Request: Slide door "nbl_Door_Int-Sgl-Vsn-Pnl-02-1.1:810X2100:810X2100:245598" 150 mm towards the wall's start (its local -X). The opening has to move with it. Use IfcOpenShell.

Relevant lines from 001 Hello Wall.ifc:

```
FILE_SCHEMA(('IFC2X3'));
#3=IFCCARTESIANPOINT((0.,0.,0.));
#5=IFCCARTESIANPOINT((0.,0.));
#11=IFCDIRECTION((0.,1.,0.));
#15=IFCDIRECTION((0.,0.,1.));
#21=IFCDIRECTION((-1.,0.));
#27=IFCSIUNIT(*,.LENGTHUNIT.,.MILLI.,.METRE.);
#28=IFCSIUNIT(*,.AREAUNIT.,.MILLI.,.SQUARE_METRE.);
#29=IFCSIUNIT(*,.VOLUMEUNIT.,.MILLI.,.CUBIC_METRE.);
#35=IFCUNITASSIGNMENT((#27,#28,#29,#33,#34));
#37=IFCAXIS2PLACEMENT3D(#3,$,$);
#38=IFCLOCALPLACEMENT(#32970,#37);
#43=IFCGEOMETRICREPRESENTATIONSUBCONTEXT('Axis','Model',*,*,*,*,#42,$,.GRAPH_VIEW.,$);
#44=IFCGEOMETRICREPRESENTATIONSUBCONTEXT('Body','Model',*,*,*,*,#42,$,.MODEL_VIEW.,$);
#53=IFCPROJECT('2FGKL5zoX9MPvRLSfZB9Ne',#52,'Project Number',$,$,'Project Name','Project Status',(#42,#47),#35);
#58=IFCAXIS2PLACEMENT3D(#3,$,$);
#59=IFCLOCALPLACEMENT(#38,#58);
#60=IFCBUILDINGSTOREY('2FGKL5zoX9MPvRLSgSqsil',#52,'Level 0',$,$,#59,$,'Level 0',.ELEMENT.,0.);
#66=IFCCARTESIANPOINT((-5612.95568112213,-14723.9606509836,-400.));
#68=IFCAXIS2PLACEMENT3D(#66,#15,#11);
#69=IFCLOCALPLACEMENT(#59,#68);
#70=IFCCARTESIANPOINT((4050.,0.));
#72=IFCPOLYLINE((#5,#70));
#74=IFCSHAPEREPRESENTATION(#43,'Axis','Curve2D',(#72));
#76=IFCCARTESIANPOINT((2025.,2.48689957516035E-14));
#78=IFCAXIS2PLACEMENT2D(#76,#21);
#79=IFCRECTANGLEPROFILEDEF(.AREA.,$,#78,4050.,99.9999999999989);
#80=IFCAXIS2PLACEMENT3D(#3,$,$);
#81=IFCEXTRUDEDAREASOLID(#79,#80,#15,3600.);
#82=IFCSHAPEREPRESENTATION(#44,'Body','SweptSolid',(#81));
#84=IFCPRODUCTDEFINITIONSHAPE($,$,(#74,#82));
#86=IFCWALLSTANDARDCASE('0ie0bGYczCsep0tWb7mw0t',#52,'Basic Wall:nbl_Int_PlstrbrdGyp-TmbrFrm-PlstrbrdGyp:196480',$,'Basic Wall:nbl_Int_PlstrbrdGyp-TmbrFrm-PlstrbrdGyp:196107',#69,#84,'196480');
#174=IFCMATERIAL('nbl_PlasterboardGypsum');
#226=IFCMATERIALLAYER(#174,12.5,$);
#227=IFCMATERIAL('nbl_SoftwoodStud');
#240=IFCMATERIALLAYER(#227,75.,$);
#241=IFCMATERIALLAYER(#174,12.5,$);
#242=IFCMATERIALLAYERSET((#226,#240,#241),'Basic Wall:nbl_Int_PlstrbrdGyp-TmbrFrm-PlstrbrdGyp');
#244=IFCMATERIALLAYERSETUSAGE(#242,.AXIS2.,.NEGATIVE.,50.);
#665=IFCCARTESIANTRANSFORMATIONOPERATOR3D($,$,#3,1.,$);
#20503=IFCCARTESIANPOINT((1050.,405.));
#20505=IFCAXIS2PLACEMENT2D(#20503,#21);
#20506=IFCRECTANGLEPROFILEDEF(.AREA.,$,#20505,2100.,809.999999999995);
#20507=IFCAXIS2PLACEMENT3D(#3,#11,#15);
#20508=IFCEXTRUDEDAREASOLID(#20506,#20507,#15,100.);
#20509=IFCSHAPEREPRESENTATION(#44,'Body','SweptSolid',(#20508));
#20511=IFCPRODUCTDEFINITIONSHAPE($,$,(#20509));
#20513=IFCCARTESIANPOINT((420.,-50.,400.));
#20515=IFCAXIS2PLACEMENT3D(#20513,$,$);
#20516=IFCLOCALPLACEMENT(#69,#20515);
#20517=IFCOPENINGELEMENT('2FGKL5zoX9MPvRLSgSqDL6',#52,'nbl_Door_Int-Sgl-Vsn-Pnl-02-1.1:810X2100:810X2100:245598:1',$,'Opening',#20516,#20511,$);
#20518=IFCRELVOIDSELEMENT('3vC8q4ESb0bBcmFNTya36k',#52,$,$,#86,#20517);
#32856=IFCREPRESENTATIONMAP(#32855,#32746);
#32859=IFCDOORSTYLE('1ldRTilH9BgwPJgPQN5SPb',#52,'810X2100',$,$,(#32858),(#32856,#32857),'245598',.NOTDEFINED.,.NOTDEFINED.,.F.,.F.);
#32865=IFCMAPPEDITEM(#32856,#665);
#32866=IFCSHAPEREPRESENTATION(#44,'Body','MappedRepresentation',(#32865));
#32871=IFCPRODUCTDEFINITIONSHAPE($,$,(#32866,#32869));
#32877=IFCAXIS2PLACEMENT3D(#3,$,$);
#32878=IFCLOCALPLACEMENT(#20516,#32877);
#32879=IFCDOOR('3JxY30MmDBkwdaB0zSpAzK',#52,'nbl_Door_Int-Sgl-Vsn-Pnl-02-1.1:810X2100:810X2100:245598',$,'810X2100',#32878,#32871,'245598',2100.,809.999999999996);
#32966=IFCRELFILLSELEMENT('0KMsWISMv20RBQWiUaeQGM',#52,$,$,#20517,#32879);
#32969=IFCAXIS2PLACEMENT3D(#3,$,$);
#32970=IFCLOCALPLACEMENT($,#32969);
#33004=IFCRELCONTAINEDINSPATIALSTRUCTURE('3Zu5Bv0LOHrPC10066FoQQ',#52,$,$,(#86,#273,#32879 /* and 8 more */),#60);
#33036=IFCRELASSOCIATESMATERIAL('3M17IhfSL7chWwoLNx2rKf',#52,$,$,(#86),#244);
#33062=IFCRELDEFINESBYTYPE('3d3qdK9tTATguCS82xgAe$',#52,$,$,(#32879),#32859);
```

```python
import ifcopenshell
import ifcopenshell.api.geometry
import ifcopenshell.util.placement

model = ifcopenshell.open("001 Hello Wall.ifc")

door = model.by_guid("3JxY30MmDBkwdaB0zSpAzK")
opening = door.FillsVoids[0].RelatingOpeningElement
wall = opening.VoidsElements[0].RelatingBuildingElement

wall_matrix = ifcopenshell.util.placement.get_local_placement(wall.ObjectPlacement)
shift = wall_matrix[:3, 0] * -150.0
before = ifcopenshell.util.placement.get_local_placement(door.ObjectPlacement)[:3, 3].copy()

# The door is placed relative to its opening, so it follows when the opening moves.
matrix = ifcopenshell.util.placement.get_local_placement(opening.ObjectPlacement)
matrix[:3, 3] += shift
ifcopenshell.api.geometry.edit_object_placement(
    model, product=opening, matrix=matrix, is_si=False, should_transform_children=True
)

after = ifcopenshell.util.placement.get_local_placement(door.ObjectPlacement)[:3, 3]
print("door moved by", (after - before).round(3) + 0.0)

model.write("001 Hello Wall-out.ifc")
```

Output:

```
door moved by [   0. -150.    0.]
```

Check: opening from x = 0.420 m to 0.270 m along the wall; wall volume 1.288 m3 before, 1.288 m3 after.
